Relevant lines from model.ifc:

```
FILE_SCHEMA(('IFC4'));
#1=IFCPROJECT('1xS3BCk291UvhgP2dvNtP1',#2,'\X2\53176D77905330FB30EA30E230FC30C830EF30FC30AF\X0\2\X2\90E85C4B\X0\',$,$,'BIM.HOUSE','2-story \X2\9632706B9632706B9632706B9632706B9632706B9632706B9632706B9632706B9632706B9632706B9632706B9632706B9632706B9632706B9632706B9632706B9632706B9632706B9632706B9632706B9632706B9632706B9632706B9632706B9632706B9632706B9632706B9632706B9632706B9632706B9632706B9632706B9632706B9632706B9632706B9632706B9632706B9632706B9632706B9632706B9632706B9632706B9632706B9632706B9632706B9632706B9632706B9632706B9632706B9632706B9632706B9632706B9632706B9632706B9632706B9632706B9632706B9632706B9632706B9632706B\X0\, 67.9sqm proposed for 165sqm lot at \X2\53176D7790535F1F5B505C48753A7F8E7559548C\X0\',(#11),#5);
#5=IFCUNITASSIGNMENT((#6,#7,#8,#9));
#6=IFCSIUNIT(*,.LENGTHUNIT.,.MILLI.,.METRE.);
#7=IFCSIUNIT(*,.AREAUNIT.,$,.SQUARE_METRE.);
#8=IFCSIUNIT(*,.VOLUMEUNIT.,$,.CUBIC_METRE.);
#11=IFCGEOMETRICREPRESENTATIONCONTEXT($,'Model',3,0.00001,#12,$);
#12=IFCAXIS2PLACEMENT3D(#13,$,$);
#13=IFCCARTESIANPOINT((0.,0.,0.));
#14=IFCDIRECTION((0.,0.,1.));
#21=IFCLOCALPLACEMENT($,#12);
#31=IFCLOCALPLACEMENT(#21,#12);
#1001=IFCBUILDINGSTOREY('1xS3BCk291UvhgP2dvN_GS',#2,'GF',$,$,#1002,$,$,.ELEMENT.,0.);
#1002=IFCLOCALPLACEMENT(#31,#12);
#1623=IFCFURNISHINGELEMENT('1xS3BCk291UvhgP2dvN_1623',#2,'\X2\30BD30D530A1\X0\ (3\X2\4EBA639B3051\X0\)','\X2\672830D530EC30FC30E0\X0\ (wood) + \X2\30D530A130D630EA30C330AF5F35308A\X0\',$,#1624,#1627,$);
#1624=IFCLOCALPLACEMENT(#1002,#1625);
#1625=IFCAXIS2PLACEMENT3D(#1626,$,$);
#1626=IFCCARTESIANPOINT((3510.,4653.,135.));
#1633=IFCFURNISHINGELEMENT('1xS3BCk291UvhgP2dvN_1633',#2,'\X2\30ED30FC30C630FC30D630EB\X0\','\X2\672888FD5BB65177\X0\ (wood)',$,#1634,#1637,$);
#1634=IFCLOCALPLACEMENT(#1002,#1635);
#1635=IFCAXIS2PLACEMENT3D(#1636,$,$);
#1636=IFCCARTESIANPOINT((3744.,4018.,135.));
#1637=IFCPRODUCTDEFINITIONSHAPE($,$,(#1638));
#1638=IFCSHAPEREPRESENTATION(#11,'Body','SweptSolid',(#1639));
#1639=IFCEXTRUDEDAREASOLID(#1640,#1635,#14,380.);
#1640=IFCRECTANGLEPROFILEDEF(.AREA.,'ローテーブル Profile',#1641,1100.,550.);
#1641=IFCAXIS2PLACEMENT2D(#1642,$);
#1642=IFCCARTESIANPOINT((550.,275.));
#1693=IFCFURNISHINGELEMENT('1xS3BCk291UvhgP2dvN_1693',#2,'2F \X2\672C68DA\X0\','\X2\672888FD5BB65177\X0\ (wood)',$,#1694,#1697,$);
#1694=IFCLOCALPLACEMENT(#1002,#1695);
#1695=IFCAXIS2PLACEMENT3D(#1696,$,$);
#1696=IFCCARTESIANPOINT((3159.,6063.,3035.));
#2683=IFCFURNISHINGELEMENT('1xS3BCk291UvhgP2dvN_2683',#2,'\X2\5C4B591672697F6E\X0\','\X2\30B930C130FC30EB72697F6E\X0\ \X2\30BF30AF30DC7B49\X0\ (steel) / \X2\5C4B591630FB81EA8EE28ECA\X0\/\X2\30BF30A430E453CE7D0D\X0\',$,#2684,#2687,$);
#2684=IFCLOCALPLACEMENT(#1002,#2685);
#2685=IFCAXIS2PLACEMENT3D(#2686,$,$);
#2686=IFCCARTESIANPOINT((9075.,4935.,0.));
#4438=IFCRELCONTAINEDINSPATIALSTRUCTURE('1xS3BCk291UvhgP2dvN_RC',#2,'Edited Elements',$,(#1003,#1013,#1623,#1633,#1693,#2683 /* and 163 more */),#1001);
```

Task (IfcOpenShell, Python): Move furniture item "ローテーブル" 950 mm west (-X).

```python
import ifcopenshell
import ifcopenshell.api.geometry
import ifcopenshell.util.placement
import ifcopenshell.util.unit

model = ifcopenshell.open("model.ifc")
unit_scale = ifcopenshell.util.unit.calculate_unit_scale(model)

item = model.by_guid("1xS3BCk291UvhgP2dvN_1633")
matrix = ifcopenshell.util.placement.get_local_placement(item.ObjectPlacement)
matrix[0, 3] -= 0.95 / unit_scale
ifcopenshell.api.geometry.edit_object_placement(model, product=item, matrix=matrix, is_si=False)

print(ifcopenshell.util.placement.get_local_placement(item.ObjectPlacement).round(3) + 0.0)

model.write("model_v2.ifc")
```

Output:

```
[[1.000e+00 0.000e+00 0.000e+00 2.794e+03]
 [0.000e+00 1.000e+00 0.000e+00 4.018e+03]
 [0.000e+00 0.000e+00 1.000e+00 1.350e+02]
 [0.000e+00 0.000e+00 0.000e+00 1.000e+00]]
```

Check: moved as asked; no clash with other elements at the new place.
